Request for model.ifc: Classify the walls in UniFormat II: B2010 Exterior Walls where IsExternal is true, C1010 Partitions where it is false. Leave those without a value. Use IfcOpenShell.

First a look at what the model holds.

```python
import ifcopenshell
import ifcopenshell.util.element

model = ifcopenshell.open("model.ifc")
print(model.schema)
print("classifications:", [c.Name for c in model.by_type("IfcClassification")])
values = [ifcopenshell.util.element.get_pset(e, "Pset_WallCommon", "IsExternal") for e in model.by_type("IfcWall")]
for value in (True, False, None):
    print("IsExternal", value, values.count(value))
```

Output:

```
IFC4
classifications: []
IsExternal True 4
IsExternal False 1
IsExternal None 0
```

```python
import ifcopenshell
import ifcopenshell.api.classification
import ifcopenshell.util.element

model = ifcopenshell.open("model.ifc")

system = ifcopenshell.api.classification.add_classification(model, classification="UniFormat II")

walls = model.by_type("IfcWall")
external = {e: ifcopenshell.util.element.get_pset(e, "Pset_WallCommon", "IsExternal") for e in walls}
for flag, code, name in ((True, "B2010", "Exterior Walls"), (False, "C1010", "Partitions")):
    products = [e for e in walls if external[e] is flag]
    ifcopenshell.api.classification.add_reference(
        model, products=products, classification=system, identification=code, name=name
    )
    print(code, len(products))

model.write("model-out.ifc")
```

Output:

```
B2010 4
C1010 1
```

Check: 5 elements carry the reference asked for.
